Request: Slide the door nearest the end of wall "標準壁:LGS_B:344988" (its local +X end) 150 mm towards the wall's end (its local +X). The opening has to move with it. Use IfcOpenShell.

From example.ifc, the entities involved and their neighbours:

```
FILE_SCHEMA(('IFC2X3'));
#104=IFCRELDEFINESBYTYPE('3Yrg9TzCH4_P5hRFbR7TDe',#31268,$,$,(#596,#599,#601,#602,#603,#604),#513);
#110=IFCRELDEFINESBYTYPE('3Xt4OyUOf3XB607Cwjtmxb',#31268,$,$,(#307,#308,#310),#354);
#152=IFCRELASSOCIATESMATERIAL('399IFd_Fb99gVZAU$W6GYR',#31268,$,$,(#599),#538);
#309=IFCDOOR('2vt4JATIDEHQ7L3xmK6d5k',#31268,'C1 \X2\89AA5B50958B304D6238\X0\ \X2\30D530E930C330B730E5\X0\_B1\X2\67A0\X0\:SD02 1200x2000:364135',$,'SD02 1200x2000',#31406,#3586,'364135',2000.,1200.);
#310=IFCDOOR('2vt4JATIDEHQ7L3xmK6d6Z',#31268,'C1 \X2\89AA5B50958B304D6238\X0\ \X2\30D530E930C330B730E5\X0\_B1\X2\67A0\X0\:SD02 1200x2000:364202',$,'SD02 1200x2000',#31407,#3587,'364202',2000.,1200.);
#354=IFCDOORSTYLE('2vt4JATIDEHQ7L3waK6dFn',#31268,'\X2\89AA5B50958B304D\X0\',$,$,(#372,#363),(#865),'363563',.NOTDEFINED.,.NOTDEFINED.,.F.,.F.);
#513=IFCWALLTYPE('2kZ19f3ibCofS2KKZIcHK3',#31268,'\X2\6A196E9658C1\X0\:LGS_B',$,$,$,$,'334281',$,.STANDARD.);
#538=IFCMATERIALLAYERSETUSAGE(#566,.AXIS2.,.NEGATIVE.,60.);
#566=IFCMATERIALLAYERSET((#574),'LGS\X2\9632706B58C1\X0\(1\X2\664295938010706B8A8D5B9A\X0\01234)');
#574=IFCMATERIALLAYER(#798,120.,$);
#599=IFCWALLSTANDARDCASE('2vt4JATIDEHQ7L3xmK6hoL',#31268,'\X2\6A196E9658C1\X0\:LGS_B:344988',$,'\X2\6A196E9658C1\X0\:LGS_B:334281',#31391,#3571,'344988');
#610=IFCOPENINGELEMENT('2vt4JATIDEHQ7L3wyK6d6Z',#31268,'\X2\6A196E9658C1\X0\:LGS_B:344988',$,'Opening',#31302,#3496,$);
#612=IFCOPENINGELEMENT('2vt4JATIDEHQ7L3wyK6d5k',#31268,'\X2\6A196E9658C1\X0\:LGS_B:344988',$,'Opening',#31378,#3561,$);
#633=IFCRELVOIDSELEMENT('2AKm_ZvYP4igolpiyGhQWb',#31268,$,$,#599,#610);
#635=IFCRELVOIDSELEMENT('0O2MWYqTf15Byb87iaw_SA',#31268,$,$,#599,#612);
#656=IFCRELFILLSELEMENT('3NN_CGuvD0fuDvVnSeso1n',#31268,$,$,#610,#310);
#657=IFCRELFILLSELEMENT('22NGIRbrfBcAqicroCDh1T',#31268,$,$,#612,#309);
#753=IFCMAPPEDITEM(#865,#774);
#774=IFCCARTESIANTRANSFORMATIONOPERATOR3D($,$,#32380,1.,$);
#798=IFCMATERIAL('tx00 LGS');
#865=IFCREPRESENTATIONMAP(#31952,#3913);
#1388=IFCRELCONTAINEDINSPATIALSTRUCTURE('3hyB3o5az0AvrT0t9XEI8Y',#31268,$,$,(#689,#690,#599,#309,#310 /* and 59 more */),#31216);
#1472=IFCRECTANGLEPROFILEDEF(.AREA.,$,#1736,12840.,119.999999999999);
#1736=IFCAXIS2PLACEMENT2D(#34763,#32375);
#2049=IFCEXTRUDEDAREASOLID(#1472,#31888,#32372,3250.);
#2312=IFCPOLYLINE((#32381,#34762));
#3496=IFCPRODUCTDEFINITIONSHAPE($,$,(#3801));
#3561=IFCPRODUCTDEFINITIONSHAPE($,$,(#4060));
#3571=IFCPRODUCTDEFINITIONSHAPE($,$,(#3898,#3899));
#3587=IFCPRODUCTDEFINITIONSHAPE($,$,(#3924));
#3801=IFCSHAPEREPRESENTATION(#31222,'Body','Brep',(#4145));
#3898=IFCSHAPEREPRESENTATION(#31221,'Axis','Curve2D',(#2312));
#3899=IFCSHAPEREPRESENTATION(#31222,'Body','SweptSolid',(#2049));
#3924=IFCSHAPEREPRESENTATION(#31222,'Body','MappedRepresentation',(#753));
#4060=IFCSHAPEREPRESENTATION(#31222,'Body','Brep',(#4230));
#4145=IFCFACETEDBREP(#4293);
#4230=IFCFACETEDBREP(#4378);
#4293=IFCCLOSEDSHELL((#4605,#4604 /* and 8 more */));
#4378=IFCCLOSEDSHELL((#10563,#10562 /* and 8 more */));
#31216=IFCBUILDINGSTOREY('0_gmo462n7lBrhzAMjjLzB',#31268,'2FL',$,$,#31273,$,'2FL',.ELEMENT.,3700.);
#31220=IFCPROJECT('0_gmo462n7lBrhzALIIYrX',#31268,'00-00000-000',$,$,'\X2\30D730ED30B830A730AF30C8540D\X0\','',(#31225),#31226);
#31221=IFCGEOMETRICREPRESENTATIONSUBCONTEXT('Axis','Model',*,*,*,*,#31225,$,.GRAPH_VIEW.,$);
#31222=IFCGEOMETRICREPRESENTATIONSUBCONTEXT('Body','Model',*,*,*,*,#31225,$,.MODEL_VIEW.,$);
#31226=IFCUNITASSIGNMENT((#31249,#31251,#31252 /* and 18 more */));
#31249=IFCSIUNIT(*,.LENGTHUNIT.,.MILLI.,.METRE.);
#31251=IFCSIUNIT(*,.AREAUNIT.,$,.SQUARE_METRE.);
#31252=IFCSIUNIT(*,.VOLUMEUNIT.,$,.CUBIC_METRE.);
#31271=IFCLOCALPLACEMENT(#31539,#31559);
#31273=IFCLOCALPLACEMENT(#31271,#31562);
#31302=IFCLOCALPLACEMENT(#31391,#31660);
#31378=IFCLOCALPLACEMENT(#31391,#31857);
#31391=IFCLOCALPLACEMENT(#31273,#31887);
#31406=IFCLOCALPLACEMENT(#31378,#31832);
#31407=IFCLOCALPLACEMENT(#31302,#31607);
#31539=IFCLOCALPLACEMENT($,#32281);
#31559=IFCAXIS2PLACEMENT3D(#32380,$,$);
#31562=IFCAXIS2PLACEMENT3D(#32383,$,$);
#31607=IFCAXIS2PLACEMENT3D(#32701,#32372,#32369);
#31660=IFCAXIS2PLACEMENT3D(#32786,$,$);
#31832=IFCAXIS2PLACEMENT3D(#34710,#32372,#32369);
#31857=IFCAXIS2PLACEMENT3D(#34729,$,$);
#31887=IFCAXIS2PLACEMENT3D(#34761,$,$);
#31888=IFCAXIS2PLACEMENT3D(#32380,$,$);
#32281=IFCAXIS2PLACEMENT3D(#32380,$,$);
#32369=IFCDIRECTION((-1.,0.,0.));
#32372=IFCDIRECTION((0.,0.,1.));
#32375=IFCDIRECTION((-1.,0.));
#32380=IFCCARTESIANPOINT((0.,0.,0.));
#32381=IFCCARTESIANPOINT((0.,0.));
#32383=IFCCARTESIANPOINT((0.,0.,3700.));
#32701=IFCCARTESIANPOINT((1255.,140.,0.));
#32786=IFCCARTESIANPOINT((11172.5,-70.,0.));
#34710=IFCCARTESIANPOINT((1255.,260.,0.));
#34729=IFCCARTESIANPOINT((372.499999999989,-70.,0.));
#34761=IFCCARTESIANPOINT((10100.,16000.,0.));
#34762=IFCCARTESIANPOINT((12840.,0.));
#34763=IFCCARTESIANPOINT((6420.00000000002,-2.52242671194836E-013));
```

```python
import ifcopenshell
import ifcopenshell.api.geometry
import ifcopenshell.util.placement
import ifcopenshell.util.unit

model = ifcopenshell.open("example.ifc")
unit_scale = ifcopenshell.util.unit.calculate_unit_scale(model)

door = model.by_guid("2vt4JATIDEHQ7L3xmK6d6Z")
opening = door.FillsVoids[0].RelatingOpeningElement
wall = opening.VoidsElements[0].RelatingBuildingElement

wall_matrix = ifcopenshell.util.placement.get_local_placement(wall.ObjectPlacement)
shift = wall_matrix[:3, 0] * 0.15 / unit_scale
before = ifcopenshell.util.placement.get_local_placement(door.ObjectPlacement)[:3, 3].copy()

# The door is placed relative to its opening, so it follows when the opening moves.
matrix = ifcopenshell.util.placement.get_local_placement(opening.ObjectPlacement)
matrix[:3, 3] += shift
ifcopenshell.api.geometry.edit_object_placement(
    model, product=opening, matrix=matrix, is_si=False, should_transform_children=True
)

after = ifcopenshell.util.placement.get_local_placement(door.ObjectPlacement)[:3, 3]
print("door moved by", (after - before).round(3) + 0.0)

model.write("example_rev.ifc")
```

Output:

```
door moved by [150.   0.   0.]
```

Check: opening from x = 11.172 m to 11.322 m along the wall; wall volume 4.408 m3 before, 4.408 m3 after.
